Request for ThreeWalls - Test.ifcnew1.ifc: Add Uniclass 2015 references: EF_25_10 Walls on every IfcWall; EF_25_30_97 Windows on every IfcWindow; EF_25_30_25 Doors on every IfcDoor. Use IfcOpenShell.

First a look at what the model holds.

```python
import ifcopenshell

model = ifcopenshell.open("ThreeWalls - Test.ifcnew1.ifc")
print(model.schema)
print("classifications:", [c.Name for c in model.by_type("IfcClassification")])
for ifc_class in ("IfcDoor", "IfcRoof", "IfcStair", "IfcWall", "IfcWindow"):
    print(ifc_class, len(model.by_type(ifc_class)))
```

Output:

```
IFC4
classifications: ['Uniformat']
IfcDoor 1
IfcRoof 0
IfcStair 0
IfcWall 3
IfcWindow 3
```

```python
import ifcopenshell
import ifcopenshell.api.classification

model = ifcopenshell.open("ThreeWalls - Test.ifcnew1.ifc")

system = ifcopenshell.api.classification.add_classification(model, classification="Uniclass 2015")

codes = {
    "IfcWall": ("EF_25_10", "Walls"),
    "IfcWindow": ("EF_25_30_97", "Windows"),
    "IfcDoor": ("EF_25_30_25", "Doors"),
}
for ifc_class, (code, name) in codes.items():
    products = model.by_type(ifc_class)
    ifcopenshell.api.classification.add_reference(
        model, products=products, classification=system, identification=code, name=name
    )
    print(code, len(products))

model.write("ThreeWalls - Test.ifcnew1_v2.ifc")
```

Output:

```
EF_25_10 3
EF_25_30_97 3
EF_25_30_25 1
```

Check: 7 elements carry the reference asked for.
